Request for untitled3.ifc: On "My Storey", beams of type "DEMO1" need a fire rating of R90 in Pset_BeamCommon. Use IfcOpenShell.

First a look at what the model holds.

```python
import ifcopenshell
import ifcopenshell.util.element

model = ifcopenshell.open("untitled3.ifc")
print(model.schema)
storey = next(s for s in model.by_type("IfcBuildingStorey") if s.Name == "My Storey")
beams = [e for e in ifcopenshell.util.element.get_decomposition(storey) if e.is_a("IfcBeam")]
seen = {}
for e in beams:
    element_type = ifcopenshell.util.element.get_type(e)
    key = (element_type.Name if element_type != e and element_type else None, ifcopenshell.util.element.get_pset(e, "Pset_BeamCommon", "FireRating"))
    seen[key] = seen.get(key, 0) + 1
for (name, value), count in sorted(seen.items(), key=str):
    print(count, "x", name, "|", value)
```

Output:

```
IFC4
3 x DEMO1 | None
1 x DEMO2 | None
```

```python
import ifcopenshell
import ifcopenshell.api.pset
import ifcopenshell.util.element

model = ifcopenshell.open("untitled3.ifc")

storey = next(s for s in model.by_type("IfcBuildingStorey") if s.Name == "My Storey")
beams = [e for e in ifcopenshell.util.element.get_decomposition(storey) if e.is_a("IfcBeam")]

count = 0
for e in beams:
    element_type = ifcopenshell.util.element.get_type(e)
    if element_type in (None, e) or element_type.Name != "DEMO1":
        continue
    # add_pset returns the element's existing set when there is one.
    pset = ifcopenshell.api.pset.add_pset(model, product=e, name="Pset_BeamCommon")
    ifcopenshell.api.pset.edit_pset(model, pset=pset, properties={"FireRating": "R90"})
    count += 1

print(count, "beams updated")

model.write("untitled3_edited.ifc")
```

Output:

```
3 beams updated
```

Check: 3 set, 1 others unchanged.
